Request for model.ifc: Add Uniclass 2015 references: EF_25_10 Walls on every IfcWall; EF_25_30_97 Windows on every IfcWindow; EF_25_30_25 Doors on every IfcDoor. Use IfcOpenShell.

First a look at what the model holds.

```python
import ifcopenshell

model = ifcopenshell.open("model.ifc")
print(model.schema)
print("classifications:", [c.Name for c in model.by_type("IfcClassification")])
for ifc_class in ("IfcDoor", "IfcRoof", "IfcStair", "IfcWall", "IfcWindow"):
    print(ifc_class, len(model.by_type(ifc_class)))
```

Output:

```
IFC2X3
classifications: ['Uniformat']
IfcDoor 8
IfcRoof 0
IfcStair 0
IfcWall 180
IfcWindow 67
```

```python
import ifcopenshell
import ifcopenshell.api.classification

model = ifcopenshell.open("model.ifc")

# IFC2X3 requires Source and Edition and has no link from the project to the system.
system = model.create_entity("IfcClassification", Source="NBS", Edition="2015", Name="Uniclass 2015")

codes = {
    "IfcWall": ("EF_25_10", "Walls"),
    "IfcWindow": ("EF_25_30_97", "Windows"),
    "IfcDoor": ("EF_25_30_25", "Doors"),
}
for ifc_class, (code, name) in codes.items():
    products = model.by_type(ifc_class)
    ifcopenshell.api.classification.add_reference(
        model, products=products, classification=system, identification=code, name=name
    )
    print(code, len(products))

model.write("model_updated.ifc")
```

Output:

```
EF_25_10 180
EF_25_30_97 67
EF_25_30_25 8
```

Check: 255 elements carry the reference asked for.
